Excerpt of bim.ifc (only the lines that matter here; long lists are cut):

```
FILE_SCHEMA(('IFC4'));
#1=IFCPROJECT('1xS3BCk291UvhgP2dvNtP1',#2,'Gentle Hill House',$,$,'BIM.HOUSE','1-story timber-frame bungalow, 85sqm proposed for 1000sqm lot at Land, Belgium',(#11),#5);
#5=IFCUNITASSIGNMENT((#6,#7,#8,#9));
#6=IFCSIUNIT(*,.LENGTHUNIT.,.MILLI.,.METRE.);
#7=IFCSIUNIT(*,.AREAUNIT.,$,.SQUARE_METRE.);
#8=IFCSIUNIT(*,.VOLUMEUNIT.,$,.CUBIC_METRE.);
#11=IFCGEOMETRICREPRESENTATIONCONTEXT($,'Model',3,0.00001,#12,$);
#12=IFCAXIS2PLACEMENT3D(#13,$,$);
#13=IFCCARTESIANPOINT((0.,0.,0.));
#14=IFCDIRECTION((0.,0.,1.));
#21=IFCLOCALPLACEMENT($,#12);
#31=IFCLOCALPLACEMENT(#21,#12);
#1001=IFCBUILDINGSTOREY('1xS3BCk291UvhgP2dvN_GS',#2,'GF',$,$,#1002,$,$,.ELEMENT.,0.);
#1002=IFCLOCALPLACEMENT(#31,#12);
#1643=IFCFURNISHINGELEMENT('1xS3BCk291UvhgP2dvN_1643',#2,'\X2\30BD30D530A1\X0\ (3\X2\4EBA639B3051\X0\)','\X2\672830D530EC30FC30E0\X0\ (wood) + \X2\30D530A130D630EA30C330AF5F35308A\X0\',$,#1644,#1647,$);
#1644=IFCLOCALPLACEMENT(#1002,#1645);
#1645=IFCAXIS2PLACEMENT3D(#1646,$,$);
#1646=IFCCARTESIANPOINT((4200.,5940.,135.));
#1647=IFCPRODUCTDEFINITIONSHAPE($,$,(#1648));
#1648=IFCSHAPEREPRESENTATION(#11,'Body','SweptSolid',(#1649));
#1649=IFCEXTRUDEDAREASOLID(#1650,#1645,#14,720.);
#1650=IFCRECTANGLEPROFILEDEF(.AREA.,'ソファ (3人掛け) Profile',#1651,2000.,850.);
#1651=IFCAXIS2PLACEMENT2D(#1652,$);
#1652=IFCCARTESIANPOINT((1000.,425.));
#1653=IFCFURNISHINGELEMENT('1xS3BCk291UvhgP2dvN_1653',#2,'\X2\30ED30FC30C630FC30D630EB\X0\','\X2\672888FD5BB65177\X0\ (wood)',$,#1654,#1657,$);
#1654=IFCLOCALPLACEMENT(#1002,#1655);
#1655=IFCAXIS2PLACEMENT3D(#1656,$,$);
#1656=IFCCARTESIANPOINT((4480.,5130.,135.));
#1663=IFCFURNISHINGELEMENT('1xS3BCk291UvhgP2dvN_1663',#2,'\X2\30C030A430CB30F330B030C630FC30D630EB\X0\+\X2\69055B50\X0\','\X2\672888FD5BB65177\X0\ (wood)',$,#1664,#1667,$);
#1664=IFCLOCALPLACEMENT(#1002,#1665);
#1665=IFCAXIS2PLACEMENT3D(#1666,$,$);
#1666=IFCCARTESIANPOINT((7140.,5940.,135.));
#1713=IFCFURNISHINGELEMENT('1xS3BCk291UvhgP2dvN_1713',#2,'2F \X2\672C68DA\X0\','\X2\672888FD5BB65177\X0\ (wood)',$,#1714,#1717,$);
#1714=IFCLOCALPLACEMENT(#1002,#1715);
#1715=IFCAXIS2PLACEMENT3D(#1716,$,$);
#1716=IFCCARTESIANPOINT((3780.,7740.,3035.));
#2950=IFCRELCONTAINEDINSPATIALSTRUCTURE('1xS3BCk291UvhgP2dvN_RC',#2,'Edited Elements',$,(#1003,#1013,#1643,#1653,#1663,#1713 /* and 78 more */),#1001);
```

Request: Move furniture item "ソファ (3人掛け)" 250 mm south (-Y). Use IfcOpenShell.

```python
import ifcopenshell
import ifcopenshell.api.geometry
import ifcopenshell.util.placement
import ifcopenshell.util.unit

model = ifcopenshell.open("bim.ifc")
unit_scale = ifcopenshell.util.unit.calculate_unit_scale(model)

item = model.by_guid("1xS3BCk291UvhgP2dvN_1643")
matrix = ifcopenshell.util.placement.get_local_placement(item.ObjectPlacement)
matrix[1, 3] -= 0.25 / unit_scale
ifcopenshell.api.geometry.edit_object_placement(model, product=item, matrix=matrix, is_si=False)

print(ifcopenshell.util.placement.get_local_placement(item.ObjectPlacement).round(3) + 0.0)

model.write("bim_rev.ifc")
```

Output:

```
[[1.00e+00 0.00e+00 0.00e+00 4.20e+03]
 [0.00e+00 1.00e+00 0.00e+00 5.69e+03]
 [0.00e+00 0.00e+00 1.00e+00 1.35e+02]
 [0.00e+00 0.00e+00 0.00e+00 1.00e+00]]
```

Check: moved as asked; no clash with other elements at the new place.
